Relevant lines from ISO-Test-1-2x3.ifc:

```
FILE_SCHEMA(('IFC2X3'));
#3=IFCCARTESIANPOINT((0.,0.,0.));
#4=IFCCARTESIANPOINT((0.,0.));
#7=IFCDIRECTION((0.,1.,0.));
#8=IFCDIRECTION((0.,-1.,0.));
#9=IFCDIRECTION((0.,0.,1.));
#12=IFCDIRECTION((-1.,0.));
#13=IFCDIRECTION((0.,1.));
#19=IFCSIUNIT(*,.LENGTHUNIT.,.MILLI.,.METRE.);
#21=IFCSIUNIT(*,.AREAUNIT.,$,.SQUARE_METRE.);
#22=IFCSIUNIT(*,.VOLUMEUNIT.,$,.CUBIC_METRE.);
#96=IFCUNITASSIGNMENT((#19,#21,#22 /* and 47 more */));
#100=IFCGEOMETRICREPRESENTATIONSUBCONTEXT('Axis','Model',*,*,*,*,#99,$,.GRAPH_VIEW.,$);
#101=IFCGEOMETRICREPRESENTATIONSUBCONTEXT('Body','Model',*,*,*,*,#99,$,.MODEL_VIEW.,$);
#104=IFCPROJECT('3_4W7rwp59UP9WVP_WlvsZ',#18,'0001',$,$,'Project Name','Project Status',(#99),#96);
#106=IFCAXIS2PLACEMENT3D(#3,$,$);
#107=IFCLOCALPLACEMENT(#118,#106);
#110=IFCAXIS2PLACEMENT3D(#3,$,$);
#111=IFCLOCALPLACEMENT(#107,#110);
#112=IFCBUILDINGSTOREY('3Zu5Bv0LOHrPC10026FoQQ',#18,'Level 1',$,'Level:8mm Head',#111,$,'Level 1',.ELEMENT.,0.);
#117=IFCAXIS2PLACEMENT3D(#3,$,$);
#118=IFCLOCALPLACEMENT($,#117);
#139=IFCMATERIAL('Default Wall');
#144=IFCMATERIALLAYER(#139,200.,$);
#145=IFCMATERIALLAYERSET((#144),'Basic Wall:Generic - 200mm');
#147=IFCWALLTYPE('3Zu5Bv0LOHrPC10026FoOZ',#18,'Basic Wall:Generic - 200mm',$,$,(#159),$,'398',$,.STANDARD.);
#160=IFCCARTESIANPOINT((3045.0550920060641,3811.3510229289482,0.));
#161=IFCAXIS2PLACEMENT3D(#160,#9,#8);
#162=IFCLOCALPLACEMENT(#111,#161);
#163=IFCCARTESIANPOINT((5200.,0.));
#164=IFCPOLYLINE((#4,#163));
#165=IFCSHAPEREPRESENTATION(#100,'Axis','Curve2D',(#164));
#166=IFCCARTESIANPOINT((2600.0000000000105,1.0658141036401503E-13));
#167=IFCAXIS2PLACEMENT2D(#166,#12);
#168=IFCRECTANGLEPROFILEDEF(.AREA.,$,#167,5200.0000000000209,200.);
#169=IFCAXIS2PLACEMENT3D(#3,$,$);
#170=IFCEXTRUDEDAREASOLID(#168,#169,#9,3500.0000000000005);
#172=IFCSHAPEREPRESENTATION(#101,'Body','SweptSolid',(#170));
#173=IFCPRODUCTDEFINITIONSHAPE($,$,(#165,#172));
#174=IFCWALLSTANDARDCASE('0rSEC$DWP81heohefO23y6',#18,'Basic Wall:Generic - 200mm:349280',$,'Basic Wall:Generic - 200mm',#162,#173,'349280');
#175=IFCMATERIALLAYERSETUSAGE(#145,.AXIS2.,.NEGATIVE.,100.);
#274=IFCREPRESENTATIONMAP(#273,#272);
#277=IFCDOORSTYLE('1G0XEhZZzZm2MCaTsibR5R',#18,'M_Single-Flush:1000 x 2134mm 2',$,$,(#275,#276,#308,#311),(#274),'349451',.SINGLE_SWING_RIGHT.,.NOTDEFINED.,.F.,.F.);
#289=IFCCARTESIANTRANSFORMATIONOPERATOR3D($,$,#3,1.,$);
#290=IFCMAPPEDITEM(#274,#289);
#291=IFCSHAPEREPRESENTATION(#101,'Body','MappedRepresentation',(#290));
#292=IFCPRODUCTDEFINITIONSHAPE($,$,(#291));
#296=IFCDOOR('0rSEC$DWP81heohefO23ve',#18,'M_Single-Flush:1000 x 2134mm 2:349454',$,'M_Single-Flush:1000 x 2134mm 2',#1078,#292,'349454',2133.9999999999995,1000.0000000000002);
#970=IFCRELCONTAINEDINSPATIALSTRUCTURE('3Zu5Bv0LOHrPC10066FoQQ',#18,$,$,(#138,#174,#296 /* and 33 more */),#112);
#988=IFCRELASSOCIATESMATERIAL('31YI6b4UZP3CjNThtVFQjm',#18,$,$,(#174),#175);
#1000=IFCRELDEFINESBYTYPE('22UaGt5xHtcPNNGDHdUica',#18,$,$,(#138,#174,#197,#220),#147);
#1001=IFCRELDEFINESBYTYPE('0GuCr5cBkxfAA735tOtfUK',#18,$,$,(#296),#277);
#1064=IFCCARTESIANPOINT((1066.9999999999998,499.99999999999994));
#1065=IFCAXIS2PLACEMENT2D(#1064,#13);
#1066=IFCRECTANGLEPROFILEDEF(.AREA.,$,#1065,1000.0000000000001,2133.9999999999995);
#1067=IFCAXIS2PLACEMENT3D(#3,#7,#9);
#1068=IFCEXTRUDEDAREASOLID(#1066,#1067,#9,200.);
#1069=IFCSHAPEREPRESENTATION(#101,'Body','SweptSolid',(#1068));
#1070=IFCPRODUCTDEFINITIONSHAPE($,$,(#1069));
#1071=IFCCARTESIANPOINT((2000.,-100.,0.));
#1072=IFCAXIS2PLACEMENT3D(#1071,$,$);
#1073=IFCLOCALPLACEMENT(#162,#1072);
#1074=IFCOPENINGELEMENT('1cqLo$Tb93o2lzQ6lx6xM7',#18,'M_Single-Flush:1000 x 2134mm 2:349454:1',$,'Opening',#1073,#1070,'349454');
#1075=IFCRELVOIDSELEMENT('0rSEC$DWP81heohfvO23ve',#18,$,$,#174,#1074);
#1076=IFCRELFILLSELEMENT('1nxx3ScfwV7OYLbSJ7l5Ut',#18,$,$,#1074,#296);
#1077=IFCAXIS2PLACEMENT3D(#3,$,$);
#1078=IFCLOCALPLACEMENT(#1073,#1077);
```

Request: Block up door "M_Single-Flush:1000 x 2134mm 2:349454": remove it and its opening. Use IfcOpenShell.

```python
import ifcopenshell
import ifcopenshell.api.feature
import ifcopenshell.api.root
import ifcopenshell.geom
import ifcopenshell.util.shape

model = ifcopenshell.open("ISO-Test-1-2x3.ifc")
settings = ifcopenshell.geom.settings()


def volume(element):
    """Net volume in cubic metres, openings subtracted."""
    shape = ifcopenshell.geom.create_shape(settings, element)
    return ifcopenshell.util.shape.get_volume(shape.geometry)


door = model.by_id(296)
opening = door.FillsVoids[0].RelatingOpeningElement
wall = opening.VoidsElements[0].RelatingBuildingElement
before = volume(wall)

ifcopenshell.api.root.remove_product(model, product=door)
ifcopenshell.api.feature.remove_feature(model, feature=opening)

after = volume(wall)

print(f"wall volume {before:.3f} -> {after:.3f} m3")

model.write("ISO-Test-1-2x3_v2.ifc")
```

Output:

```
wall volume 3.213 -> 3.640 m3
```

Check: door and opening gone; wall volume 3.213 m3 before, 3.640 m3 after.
